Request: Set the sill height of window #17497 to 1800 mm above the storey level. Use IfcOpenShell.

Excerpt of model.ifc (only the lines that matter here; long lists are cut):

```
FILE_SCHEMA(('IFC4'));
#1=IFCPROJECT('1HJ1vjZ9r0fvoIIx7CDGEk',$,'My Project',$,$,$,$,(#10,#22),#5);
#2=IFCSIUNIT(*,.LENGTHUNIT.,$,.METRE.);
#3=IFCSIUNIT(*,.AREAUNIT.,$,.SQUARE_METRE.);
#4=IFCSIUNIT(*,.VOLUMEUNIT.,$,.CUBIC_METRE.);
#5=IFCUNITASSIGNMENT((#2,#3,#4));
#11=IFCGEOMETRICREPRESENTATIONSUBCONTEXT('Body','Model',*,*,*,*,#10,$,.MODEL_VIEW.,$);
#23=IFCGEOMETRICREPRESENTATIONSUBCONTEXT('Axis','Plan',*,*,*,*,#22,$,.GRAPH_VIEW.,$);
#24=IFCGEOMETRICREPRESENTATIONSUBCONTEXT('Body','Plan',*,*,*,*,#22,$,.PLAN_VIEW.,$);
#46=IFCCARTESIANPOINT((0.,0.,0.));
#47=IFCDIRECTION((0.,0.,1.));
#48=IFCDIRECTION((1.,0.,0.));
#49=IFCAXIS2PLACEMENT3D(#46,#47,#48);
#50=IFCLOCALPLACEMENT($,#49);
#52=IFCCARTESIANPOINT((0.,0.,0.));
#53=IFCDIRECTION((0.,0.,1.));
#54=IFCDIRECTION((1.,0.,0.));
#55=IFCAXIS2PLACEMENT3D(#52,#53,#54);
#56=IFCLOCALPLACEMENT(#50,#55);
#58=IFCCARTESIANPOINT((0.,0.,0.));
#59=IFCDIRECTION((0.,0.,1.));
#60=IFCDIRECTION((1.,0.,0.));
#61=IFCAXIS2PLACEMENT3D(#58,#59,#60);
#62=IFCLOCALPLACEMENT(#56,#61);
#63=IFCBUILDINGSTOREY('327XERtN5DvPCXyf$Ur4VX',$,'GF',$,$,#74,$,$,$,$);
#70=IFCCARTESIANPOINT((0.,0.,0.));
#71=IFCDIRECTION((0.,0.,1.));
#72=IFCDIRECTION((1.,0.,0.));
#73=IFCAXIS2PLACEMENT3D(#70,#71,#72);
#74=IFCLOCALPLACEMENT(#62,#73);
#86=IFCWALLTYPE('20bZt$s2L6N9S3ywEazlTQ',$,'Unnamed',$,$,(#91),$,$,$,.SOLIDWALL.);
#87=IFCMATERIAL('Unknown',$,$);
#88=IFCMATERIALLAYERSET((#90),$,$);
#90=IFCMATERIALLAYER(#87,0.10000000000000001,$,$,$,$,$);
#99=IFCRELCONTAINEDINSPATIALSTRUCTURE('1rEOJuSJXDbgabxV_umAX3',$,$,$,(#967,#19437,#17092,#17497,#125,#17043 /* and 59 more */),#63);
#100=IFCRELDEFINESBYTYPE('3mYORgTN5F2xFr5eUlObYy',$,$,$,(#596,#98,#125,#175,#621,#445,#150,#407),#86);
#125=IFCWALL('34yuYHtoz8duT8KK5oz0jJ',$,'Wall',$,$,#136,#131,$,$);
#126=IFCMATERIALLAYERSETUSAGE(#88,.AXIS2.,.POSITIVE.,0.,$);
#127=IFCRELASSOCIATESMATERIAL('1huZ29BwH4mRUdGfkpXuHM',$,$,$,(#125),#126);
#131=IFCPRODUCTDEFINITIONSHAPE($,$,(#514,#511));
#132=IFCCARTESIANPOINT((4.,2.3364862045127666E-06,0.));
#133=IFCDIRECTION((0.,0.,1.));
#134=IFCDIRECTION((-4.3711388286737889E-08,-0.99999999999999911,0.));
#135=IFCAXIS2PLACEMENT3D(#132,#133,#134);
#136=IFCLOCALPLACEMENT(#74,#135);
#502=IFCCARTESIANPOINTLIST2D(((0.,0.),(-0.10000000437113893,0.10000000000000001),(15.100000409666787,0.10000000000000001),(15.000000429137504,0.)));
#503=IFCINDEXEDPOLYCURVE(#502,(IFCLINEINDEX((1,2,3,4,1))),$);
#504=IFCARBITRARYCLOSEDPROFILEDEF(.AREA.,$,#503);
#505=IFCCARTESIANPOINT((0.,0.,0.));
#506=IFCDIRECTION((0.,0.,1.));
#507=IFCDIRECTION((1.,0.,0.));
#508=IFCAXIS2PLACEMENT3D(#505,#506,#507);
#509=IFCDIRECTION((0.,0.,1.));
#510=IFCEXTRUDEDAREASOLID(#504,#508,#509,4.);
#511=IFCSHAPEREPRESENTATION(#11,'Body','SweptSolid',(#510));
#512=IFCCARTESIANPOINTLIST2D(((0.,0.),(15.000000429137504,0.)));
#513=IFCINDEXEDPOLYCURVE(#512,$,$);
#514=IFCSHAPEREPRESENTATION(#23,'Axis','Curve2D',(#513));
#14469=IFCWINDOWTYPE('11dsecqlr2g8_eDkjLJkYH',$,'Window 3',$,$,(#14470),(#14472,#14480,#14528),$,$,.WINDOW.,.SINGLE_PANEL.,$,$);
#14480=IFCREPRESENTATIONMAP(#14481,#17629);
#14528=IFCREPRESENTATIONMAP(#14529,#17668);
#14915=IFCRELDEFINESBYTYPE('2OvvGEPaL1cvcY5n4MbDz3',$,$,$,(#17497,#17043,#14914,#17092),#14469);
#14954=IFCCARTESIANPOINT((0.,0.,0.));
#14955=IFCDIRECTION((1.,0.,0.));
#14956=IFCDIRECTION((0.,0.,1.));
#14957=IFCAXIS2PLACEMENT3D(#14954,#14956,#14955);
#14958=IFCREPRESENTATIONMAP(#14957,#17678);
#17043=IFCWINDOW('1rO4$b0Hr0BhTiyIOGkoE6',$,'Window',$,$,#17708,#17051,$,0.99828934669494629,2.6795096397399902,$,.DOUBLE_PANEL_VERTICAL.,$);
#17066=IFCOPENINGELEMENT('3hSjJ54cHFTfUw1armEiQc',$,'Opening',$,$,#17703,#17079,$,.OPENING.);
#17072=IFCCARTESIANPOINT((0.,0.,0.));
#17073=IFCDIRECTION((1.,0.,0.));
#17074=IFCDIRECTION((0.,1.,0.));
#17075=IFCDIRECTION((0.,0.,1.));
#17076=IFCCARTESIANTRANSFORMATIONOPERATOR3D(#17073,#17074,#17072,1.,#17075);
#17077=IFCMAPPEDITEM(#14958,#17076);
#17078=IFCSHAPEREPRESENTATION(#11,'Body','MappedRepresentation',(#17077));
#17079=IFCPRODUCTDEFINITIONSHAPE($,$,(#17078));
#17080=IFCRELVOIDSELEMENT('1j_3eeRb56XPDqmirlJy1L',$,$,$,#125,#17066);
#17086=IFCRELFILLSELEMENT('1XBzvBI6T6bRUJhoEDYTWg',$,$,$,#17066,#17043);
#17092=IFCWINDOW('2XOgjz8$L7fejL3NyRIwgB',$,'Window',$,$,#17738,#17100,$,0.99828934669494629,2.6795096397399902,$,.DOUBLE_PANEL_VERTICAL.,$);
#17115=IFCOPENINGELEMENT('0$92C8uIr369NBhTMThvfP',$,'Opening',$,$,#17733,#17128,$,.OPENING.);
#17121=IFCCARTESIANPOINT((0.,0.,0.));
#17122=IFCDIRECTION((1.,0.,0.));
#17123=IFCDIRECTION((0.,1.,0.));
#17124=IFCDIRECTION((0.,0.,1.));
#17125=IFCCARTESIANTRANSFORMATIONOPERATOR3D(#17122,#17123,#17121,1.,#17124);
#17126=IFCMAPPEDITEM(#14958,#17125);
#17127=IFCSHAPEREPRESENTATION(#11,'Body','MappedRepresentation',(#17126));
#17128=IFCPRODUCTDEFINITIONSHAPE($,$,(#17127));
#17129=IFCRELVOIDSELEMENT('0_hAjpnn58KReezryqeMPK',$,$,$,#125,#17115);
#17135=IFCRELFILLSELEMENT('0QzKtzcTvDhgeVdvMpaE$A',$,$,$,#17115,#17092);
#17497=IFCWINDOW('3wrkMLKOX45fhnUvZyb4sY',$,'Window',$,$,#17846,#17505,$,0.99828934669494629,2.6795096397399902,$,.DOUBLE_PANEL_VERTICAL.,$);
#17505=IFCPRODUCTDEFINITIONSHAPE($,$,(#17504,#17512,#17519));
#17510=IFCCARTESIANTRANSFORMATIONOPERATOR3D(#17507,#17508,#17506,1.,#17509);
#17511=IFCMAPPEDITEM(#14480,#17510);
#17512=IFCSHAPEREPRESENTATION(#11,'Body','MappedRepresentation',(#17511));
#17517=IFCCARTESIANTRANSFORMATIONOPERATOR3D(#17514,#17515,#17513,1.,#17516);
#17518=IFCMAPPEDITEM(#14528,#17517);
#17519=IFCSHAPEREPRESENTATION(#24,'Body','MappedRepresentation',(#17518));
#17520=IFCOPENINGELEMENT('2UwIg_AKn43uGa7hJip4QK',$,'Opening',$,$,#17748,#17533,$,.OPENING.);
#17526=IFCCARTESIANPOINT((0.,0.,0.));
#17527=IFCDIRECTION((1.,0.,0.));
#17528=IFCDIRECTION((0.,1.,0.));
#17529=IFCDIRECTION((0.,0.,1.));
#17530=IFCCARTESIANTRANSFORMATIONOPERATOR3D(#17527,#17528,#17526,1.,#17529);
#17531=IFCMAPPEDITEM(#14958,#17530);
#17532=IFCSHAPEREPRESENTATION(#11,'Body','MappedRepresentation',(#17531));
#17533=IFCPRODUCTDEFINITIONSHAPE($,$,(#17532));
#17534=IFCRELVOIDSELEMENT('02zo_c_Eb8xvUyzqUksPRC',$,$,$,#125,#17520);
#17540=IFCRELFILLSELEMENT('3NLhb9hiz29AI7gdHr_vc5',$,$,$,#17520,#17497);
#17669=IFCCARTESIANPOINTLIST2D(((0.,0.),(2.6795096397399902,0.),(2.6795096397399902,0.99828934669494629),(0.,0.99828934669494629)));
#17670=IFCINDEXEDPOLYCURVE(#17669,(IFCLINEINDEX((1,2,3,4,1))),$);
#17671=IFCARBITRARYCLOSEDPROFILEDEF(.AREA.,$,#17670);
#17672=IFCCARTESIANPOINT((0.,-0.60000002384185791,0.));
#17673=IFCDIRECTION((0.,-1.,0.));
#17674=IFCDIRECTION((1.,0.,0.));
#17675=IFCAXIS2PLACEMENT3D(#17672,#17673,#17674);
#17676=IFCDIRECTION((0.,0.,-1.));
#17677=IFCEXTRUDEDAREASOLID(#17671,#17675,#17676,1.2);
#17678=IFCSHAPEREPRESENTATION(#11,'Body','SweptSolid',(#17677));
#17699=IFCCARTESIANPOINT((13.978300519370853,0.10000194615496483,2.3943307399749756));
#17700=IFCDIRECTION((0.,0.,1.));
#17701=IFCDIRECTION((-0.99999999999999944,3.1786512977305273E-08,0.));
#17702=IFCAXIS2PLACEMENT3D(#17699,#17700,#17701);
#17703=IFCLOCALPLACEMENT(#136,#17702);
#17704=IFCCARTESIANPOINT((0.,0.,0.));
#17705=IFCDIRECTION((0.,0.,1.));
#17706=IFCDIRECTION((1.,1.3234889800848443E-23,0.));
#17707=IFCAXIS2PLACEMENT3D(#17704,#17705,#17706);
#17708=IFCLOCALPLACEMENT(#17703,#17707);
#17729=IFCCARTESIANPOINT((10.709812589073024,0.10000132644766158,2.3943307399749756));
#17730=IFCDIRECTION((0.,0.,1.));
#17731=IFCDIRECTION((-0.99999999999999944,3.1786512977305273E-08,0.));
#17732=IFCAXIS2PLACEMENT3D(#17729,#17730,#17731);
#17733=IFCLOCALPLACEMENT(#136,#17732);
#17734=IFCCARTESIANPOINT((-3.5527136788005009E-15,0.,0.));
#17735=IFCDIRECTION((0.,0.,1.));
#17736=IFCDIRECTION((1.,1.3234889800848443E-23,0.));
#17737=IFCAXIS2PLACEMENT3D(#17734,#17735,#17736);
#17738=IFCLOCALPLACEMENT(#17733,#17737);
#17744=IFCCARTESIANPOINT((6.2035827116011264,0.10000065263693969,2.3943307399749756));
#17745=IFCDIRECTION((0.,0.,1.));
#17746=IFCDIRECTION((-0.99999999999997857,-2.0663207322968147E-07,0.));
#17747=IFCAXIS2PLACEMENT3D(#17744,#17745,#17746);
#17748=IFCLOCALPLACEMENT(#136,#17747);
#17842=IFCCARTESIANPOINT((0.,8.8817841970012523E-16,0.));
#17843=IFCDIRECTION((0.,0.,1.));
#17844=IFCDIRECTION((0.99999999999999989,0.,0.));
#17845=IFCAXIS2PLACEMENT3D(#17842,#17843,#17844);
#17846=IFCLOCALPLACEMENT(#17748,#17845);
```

```python
import numpy as np
import ifcopenshell
import ifcopenshell.api.geometry
import ifcopenshell.geom
import ifcopenshell.util.element
import ifcopenshell.util.placement
import ifcopenshell.util.shape
import ifcopenshell.util.unit

model = ifcopenshell.open("model.ifc")
unit_scale = ifcopenshell.util.unit.calculate_unit_scale(model)

window = model.by_guid("3wrkMLKOX45fhnUvZyb4sY")
opening = window.FillsVoids[0].RelatingOpeningElement
storey = ifcopenshell.util.element.get_container(window, ifc_class="IfcBuildingStorey")
level = ifcopenshell.util.placement.get_local_placement(storey.ObjectPlacement)[2, 3]

# The opening's origin need not be at the sill, so measure its lowest point.
shape = ifcopenshell.geom.create_shape(ifcopenshell.geom.settings(), opening)
bottom = ifcopenshell.util.shape.get_shape_bottom_elevation(shape, shape.geometry) / unit_scale
dz = level + 1.8 / unit_scale - bottom

shift = np.array([0.0, 0.0, dz])
# The window is placed relative to its opening, so it follows when the opening moves.
matrix = ifcopenshell.util.placement.get_local_placement(opening.ObjectPlacement)
matrix[:3, 3] += shift
ifcopenshell.api.geometry.edit_object_placement(
    model, product=opening, matrix=matrix, is_si=False, should_transform_children=True
)

print(f"moved by {dz * unit_scale:+.3f} m")

model.write("model_edited.ifc")
```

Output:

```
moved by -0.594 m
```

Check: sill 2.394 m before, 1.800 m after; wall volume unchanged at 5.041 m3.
